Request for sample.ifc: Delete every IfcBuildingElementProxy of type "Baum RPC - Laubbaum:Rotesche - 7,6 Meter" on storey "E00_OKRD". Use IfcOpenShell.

First a look at what the model holds.

```python
import ifcopenshell
import ifcopenshell.util.element

model = ifcopenshell.open("sample.ifc")
print(model.schema)
storey = next(s for s in model.by_type("IfcBuildingStorey") if s.Name == "E00_OKRD")
proxies = [e for e in ifcopenshell.util.element.get_decomposition(storey) if e.is_a("IfcBuildingElementProxy")]
seen = {}
for e in proxies:
    element_type = ifcopenshell.util.element.get_type(e)
    name = element_type.Name if element_type not in (None, e) else None
    seen[name] = seen.get(name, 0) + 1
for name, count in sorted(seen.items(), key=str):
    print(count, "x", name)
```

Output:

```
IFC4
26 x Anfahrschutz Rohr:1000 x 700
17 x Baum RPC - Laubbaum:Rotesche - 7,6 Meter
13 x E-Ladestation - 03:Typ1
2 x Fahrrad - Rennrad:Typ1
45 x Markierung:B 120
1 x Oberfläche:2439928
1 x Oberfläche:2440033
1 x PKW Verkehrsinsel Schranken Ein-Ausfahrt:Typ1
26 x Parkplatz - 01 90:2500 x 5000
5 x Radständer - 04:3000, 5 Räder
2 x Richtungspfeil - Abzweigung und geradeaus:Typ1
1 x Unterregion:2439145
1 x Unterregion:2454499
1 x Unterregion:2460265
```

```python
import ifcopenshell
import ifcopenshell.api.root
import ifcopenshell.util.element

model = ifcopenshell.open("sample.ifc")

storey = next(s for s in model.by_type("IfcBuildingStorey") if s.Name == "E00_OKRD")
proxies = [e for e in ifcopenshell.util.element.get_decomposition(storey) if e.is_a("IfcBuildingElementProxy")]
targets = [e for e in proxies if (t := ifcopenshell.util.element.get_type(e)) not in (None, e) and t.Name == "Baum RPC - Laubbaum:Rotesche - 7,6 Meter"]

for e in targets:
    ifcopenshell.api.root.remove_product(model, product=e)
print(len(targets), "removed")

model.write("sample_rev.ifc")
```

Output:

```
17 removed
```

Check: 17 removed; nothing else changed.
